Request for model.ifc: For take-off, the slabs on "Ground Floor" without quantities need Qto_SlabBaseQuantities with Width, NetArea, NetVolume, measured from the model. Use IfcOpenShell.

First a look at what the model holds.

```python
import ifcopenshell
import ifcopenshell.util.element
import ifcopenshell.util.unit

model = ifcopenshell.open("model.ifc")
print(model.schema)
for unit_type in ("LENGTHUNIT", "AREAUNIT", "VOLUMEUNIT"):
    print(unit_type, ifcopenshell.util.unit.calculate_unit_scale(model, unit_type))
storey = next(s for s in model.by_type("IfcBuildingStorey") if s.Name == "Ground Floor")
slabs = [e for e in ifcopenshell.util.element.get_decomposition(storey) if e.is_a("IfcSlab")]
for e in sorted(slabs, key=lambda e: e.id()):
    print(e.id(), e.is_a(), e.Name, list(ifcopenshell.util.element.get_psets(e, qtos_only=True)), sep=" | ")
```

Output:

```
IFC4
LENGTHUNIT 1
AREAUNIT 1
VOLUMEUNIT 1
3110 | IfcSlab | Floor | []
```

```python
import ifcopenshell
import ifcopenshell.api.pset
import ifcopenshell.geom
import ifcopenshell.util.element
import ifcopenshell.util.shape
import ifcopenshell.util.unit

model = ifcopenshell.open("model.ifc")
unit_scale = ifcopenshell.util.unit.calculate_unit_scale(model)
area_scale = ifcopenshell.util.unit.calculate_unit_scale(model, "AREAUNIT")
volume_scale = ifcopenshell.util.unit.calculate_unit_scale(model, "VOLUMEUNIT")
settings = ifcopenshell.geom.settings()

storey = next(s for s in model.by_type("IfcBuildingStorey") if s.Name == "Ground Floor")
slabs = [e for e in ifcopenshell.util.element.get_decomposition(storey) if e.is_a("IfcSlab")]

for e in sorted(slabs, key=lambda e: e.id()):
    if ifcopenshell.util.element.get_psets(e, qtos_only=True, should_inherit=False):
        continue
    # Geometry comes back in metres, in the element's own axes.
    shape = ifcopenshell.geom.create_shape(settings, e)
    values = {
        "Width": ifcopenshell.util.shape.get_z(shape.geometry) / unit_scale,
        "NetArea": ifcopenshell.util.shape.get_footprint_area(shape.geometry) / area_scale,
        "NetVolume": ifcopenshell.util.shape.get_volume(shape.geometry) / volume_scale,
    }
    qto = ifcopenshell.api.pset.add_qto(model, product=e, name="Qto_SlabBaseQuantities")
    ifcopenshell.api.pset.edit_qto(model, qto=qto, properties=values)
    print(e.id(), {k: round(v, 3) for k, v in values.items()})

model.write("model_v2.ifc")
```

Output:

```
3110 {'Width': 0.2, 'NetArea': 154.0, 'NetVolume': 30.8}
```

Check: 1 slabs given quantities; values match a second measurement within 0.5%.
